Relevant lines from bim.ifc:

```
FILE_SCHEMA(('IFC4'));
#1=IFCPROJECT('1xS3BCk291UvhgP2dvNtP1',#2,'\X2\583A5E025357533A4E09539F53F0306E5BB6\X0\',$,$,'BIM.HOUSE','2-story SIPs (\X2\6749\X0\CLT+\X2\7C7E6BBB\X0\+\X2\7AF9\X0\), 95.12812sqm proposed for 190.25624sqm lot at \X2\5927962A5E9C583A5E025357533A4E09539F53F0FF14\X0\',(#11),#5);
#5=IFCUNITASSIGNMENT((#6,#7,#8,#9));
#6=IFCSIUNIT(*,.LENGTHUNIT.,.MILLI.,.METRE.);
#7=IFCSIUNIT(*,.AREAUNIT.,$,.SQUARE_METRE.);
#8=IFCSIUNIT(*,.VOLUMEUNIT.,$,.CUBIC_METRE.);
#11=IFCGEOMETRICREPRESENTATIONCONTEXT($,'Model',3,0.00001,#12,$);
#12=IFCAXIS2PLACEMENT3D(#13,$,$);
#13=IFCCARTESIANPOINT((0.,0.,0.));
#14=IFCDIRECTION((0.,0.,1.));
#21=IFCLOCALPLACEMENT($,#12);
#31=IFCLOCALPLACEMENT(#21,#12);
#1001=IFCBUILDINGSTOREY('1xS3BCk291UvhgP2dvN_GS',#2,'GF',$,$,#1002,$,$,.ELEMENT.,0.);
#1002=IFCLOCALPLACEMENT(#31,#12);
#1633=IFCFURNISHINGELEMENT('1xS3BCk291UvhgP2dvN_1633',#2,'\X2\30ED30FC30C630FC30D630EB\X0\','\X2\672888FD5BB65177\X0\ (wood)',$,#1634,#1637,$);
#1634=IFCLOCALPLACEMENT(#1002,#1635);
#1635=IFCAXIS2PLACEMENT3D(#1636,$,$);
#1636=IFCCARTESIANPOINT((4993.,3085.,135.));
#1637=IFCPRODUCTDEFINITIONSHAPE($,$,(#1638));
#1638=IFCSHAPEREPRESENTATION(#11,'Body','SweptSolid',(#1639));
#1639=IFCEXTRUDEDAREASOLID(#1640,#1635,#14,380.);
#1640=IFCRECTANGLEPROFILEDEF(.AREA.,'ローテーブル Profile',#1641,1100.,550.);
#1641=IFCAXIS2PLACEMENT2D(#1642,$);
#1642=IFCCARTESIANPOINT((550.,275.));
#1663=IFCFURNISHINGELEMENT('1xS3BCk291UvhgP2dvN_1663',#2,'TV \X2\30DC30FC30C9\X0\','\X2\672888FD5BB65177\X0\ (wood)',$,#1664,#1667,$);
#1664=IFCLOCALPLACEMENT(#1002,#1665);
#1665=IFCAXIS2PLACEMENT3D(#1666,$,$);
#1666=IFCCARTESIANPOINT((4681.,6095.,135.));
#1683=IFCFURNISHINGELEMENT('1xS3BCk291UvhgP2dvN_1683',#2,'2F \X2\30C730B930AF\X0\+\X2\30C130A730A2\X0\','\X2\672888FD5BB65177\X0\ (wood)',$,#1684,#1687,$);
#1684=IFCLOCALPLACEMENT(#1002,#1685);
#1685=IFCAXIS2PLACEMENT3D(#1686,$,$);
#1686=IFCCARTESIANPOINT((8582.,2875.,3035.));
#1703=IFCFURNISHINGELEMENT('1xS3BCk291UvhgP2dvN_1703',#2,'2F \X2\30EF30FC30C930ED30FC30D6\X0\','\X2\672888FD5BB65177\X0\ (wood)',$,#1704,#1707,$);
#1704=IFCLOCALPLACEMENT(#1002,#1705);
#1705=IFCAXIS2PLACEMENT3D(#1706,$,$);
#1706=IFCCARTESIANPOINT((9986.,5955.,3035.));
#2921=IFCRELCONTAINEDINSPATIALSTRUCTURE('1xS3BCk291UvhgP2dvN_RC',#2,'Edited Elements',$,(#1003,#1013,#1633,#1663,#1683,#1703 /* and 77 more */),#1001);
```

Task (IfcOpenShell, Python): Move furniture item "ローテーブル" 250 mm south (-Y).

```python
import ifcopenshell
import ifcopenshell.api.geometry
import ifcopenshell.util.placement
import ifcopenshell.util.unit

model = ifcopenshell.open("bim.ifc")
unit_scale = ifcopenshell.util.unit.calculate_unit_scale(model)

item = model.by_guid("1xS3BCk291UvhgP2dvN_1633")
matrix = ifcopenshell.util.placement.get_local_placement(item.ObjectPlacement)
matrix[1, 3] -= 0.25 / unit_scale
ifcopenshell.api.geometry.edit_object_placement(model, product=item, matrix=matrix, is_si=False)

print(ifcopenshell.util.placement.get_local_placement(item.ObjectPlacement).round(3) + 0.0)

model.write("bim-out.ifc")
```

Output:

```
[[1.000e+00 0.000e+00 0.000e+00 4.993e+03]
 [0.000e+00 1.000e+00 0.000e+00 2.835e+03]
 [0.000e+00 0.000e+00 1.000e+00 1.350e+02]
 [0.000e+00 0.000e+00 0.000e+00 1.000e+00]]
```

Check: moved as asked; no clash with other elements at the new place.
